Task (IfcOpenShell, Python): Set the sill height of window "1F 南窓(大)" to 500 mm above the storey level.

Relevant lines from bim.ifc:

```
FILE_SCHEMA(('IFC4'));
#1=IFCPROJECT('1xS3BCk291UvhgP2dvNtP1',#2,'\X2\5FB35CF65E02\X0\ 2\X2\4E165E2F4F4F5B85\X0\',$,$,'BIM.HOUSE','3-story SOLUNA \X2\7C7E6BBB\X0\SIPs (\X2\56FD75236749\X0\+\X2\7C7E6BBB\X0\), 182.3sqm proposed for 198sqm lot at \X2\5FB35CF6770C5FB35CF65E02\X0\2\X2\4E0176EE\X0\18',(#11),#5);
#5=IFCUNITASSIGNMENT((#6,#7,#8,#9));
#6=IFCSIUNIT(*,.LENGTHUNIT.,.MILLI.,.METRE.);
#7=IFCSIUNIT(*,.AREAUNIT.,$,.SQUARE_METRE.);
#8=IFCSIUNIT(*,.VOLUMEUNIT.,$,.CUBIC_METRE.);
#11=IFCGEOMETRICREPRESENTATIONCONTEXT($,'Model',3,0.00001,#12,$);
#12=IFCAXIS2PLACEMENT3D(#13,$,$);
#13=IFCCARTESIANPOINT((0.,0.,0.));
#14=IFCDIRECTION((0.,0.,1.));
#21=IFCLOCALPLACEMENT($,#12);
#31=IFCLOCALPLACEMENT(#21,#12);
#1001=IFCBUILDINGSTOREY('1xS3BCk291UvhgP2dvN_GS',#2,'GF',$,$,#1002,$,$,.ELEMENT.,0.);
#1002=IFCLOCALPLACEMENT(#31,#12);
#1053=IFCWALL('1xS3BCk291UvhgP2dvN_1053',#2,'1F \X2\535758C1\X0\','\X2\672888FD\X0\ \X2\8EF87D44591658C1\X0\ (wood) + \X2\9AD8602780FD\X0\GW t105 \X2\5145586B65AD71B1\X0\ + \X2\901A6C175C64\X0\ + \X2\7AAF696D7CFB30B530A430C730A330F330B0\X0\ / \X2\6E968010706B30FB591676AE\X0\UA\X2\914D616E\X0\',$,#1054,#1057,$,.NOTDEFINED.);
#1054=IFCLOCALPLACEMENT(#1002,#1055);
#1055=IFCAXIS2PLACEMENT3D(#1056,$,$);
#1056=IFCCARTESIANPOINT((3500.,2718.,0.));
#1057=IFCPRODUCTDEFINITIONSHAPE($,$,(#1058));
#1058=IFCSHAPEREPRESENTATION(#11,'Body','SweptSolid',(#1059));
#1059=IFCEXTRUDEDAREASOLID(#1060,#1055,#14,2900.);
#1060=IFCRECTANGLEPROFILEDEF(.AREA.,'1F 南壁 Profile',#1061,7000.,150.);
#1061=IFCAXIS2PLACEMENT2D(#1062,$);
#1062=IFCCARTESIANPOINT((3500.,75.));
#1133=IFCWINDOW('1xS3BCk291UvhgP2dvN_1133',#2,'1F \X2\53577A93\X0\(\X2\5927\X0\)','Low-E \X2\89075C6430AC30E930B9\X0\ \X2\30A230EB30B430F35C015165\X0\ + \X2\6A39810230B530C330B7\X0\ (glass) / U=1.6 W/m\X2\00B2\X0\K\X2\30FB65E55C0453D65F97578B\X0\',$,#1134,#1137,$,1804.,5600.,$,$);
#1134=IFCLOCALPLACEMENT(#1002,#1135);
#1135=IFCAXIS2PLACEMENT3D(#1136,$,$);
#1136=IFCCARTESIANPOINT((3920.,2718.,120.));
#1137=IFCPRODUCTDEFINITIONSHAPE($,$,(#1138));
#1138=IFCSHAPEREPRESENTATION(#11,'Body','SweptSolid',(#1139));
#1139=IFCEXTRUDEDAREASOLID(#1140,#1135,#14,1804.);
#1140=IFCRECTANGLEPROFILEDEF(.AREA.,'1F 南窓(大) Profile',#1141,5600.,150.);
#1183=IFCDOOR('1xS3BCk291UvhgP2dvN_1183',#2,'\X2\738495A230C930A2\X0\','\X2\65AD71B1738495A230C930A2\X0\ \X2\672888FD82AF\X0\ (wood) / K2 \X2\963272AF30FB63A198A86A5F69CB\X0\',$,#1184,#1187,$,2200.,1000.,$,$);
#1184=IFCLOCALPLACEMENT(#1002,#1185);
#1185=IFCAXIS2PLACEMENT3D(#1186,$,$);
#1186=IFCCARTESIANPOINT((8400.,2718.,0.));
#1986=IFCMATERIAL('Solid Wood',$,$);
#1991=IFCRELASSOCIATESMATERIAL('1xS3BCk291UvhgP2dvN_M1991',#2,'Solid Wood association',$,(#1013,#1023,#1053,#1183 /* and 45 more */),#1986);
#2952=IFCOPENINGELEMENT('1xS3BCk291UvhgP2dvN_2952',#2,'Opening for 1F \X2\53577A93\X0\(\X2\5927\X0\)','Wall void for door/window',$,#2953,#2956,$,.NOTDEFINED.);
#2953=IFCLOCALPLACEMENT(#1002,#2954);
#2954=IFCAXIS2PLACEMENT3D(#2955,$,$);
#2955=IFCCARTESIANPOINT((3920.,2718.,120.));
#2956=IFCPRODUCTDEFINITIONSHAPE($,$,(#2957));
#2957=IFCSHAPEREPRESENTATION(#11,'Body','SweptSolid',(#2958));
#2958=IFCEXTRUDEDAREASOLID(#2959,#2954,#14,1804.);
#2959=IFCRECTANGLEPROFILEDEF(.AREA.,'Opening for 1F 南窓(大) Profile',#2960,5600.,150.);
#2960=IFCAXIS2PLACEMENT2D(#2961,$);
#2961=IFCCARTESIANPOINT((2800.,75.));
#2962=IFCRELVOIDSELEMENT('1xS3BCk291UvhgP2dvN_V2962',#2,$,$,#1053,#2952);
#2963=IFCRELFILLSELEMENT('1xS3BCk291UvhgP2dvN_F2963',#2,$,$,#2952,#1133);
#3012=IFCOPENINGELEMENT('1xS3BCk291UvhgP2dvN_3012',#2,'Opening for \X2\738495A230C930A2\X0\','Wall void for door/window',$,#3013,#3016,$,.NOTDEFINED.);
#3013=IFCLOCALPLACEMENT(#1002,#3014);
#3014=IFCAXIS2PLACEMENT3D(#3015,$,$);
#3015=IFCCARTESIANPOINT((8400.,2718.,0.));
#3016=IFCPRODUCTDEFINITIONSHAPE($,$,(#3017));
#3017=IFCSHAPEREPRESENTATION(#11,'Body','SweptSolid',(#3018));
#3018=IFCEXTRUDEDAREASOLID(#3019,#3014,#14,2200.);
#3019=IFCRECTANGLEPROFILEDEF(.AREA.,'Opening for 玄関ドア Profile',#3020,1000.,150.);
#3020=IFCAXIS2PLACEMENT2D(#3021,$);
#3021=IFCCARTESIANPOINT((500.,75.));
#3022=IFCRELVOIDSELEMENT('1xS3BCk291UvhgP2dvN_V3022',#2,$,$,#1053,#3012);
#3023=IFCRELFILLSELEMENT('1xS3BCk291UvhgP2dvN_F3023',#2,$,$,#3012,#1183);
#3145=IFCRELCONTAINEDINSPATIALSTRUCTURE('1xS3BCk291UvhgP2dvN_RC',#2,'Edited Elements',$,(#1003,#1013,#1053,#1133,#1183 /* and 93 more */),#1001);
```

```python
import numpy as np
import ifcopenshell
import ifcopenshell.api.geometry
import ifcopenshell.geom
import ifcopenshell.util.element
import ifcopenshell.util.placement
import ifcopenshell.util.shape
import ifcopenshell.util.unit

model = ifcopenshell.open("bim.ifc")
unit_scale = ifcopenshell.util.unit.calculate_unit_scale(model)

window = model.by_guid("1xS3BCk291UvhgP2dvN_1133")
opening = window.FillsVoids[0].RelatingOpeningElement
storey = ifcopenshell.util.element.get_container(window, ifc_class="IfcBuildingStorey")
level = ifcopenshell.util.placement.get_local_placement(storey.ObjectPlacement)[2, 3]

# The opening's origin need not be at the sill, so measure its lowest point.
shape = ifcopenshell.geom.create_shape(ifcopenshell.geom.settings(), opening)
bottom = ifcopenshell.util.shape.get_shape_bottom_elevation(shape, shape.geometry) / unit_scale
dz = level + 0.5 / unit_scale - bottom

shift = np.array([0.0, 0.0, dz])
# The window is not placed relative to its opening, so move both.
for product in (opening, window):
    matrix = ifcopenshell.util.placement.get_local_placement(product.ObjectPlacement)
    matrix[:3, 3] += shift
    ifcopenshell.api.geometry.edit_object_placement(model, product=product, matrix=matrix, is_si=False)

print(f"moved by {dz * unit_scale:+.3f} m")

model.write("bim_rev.ifc")
```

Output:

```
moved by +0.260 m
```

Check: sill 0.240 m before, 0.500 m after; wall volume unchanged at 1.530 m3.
